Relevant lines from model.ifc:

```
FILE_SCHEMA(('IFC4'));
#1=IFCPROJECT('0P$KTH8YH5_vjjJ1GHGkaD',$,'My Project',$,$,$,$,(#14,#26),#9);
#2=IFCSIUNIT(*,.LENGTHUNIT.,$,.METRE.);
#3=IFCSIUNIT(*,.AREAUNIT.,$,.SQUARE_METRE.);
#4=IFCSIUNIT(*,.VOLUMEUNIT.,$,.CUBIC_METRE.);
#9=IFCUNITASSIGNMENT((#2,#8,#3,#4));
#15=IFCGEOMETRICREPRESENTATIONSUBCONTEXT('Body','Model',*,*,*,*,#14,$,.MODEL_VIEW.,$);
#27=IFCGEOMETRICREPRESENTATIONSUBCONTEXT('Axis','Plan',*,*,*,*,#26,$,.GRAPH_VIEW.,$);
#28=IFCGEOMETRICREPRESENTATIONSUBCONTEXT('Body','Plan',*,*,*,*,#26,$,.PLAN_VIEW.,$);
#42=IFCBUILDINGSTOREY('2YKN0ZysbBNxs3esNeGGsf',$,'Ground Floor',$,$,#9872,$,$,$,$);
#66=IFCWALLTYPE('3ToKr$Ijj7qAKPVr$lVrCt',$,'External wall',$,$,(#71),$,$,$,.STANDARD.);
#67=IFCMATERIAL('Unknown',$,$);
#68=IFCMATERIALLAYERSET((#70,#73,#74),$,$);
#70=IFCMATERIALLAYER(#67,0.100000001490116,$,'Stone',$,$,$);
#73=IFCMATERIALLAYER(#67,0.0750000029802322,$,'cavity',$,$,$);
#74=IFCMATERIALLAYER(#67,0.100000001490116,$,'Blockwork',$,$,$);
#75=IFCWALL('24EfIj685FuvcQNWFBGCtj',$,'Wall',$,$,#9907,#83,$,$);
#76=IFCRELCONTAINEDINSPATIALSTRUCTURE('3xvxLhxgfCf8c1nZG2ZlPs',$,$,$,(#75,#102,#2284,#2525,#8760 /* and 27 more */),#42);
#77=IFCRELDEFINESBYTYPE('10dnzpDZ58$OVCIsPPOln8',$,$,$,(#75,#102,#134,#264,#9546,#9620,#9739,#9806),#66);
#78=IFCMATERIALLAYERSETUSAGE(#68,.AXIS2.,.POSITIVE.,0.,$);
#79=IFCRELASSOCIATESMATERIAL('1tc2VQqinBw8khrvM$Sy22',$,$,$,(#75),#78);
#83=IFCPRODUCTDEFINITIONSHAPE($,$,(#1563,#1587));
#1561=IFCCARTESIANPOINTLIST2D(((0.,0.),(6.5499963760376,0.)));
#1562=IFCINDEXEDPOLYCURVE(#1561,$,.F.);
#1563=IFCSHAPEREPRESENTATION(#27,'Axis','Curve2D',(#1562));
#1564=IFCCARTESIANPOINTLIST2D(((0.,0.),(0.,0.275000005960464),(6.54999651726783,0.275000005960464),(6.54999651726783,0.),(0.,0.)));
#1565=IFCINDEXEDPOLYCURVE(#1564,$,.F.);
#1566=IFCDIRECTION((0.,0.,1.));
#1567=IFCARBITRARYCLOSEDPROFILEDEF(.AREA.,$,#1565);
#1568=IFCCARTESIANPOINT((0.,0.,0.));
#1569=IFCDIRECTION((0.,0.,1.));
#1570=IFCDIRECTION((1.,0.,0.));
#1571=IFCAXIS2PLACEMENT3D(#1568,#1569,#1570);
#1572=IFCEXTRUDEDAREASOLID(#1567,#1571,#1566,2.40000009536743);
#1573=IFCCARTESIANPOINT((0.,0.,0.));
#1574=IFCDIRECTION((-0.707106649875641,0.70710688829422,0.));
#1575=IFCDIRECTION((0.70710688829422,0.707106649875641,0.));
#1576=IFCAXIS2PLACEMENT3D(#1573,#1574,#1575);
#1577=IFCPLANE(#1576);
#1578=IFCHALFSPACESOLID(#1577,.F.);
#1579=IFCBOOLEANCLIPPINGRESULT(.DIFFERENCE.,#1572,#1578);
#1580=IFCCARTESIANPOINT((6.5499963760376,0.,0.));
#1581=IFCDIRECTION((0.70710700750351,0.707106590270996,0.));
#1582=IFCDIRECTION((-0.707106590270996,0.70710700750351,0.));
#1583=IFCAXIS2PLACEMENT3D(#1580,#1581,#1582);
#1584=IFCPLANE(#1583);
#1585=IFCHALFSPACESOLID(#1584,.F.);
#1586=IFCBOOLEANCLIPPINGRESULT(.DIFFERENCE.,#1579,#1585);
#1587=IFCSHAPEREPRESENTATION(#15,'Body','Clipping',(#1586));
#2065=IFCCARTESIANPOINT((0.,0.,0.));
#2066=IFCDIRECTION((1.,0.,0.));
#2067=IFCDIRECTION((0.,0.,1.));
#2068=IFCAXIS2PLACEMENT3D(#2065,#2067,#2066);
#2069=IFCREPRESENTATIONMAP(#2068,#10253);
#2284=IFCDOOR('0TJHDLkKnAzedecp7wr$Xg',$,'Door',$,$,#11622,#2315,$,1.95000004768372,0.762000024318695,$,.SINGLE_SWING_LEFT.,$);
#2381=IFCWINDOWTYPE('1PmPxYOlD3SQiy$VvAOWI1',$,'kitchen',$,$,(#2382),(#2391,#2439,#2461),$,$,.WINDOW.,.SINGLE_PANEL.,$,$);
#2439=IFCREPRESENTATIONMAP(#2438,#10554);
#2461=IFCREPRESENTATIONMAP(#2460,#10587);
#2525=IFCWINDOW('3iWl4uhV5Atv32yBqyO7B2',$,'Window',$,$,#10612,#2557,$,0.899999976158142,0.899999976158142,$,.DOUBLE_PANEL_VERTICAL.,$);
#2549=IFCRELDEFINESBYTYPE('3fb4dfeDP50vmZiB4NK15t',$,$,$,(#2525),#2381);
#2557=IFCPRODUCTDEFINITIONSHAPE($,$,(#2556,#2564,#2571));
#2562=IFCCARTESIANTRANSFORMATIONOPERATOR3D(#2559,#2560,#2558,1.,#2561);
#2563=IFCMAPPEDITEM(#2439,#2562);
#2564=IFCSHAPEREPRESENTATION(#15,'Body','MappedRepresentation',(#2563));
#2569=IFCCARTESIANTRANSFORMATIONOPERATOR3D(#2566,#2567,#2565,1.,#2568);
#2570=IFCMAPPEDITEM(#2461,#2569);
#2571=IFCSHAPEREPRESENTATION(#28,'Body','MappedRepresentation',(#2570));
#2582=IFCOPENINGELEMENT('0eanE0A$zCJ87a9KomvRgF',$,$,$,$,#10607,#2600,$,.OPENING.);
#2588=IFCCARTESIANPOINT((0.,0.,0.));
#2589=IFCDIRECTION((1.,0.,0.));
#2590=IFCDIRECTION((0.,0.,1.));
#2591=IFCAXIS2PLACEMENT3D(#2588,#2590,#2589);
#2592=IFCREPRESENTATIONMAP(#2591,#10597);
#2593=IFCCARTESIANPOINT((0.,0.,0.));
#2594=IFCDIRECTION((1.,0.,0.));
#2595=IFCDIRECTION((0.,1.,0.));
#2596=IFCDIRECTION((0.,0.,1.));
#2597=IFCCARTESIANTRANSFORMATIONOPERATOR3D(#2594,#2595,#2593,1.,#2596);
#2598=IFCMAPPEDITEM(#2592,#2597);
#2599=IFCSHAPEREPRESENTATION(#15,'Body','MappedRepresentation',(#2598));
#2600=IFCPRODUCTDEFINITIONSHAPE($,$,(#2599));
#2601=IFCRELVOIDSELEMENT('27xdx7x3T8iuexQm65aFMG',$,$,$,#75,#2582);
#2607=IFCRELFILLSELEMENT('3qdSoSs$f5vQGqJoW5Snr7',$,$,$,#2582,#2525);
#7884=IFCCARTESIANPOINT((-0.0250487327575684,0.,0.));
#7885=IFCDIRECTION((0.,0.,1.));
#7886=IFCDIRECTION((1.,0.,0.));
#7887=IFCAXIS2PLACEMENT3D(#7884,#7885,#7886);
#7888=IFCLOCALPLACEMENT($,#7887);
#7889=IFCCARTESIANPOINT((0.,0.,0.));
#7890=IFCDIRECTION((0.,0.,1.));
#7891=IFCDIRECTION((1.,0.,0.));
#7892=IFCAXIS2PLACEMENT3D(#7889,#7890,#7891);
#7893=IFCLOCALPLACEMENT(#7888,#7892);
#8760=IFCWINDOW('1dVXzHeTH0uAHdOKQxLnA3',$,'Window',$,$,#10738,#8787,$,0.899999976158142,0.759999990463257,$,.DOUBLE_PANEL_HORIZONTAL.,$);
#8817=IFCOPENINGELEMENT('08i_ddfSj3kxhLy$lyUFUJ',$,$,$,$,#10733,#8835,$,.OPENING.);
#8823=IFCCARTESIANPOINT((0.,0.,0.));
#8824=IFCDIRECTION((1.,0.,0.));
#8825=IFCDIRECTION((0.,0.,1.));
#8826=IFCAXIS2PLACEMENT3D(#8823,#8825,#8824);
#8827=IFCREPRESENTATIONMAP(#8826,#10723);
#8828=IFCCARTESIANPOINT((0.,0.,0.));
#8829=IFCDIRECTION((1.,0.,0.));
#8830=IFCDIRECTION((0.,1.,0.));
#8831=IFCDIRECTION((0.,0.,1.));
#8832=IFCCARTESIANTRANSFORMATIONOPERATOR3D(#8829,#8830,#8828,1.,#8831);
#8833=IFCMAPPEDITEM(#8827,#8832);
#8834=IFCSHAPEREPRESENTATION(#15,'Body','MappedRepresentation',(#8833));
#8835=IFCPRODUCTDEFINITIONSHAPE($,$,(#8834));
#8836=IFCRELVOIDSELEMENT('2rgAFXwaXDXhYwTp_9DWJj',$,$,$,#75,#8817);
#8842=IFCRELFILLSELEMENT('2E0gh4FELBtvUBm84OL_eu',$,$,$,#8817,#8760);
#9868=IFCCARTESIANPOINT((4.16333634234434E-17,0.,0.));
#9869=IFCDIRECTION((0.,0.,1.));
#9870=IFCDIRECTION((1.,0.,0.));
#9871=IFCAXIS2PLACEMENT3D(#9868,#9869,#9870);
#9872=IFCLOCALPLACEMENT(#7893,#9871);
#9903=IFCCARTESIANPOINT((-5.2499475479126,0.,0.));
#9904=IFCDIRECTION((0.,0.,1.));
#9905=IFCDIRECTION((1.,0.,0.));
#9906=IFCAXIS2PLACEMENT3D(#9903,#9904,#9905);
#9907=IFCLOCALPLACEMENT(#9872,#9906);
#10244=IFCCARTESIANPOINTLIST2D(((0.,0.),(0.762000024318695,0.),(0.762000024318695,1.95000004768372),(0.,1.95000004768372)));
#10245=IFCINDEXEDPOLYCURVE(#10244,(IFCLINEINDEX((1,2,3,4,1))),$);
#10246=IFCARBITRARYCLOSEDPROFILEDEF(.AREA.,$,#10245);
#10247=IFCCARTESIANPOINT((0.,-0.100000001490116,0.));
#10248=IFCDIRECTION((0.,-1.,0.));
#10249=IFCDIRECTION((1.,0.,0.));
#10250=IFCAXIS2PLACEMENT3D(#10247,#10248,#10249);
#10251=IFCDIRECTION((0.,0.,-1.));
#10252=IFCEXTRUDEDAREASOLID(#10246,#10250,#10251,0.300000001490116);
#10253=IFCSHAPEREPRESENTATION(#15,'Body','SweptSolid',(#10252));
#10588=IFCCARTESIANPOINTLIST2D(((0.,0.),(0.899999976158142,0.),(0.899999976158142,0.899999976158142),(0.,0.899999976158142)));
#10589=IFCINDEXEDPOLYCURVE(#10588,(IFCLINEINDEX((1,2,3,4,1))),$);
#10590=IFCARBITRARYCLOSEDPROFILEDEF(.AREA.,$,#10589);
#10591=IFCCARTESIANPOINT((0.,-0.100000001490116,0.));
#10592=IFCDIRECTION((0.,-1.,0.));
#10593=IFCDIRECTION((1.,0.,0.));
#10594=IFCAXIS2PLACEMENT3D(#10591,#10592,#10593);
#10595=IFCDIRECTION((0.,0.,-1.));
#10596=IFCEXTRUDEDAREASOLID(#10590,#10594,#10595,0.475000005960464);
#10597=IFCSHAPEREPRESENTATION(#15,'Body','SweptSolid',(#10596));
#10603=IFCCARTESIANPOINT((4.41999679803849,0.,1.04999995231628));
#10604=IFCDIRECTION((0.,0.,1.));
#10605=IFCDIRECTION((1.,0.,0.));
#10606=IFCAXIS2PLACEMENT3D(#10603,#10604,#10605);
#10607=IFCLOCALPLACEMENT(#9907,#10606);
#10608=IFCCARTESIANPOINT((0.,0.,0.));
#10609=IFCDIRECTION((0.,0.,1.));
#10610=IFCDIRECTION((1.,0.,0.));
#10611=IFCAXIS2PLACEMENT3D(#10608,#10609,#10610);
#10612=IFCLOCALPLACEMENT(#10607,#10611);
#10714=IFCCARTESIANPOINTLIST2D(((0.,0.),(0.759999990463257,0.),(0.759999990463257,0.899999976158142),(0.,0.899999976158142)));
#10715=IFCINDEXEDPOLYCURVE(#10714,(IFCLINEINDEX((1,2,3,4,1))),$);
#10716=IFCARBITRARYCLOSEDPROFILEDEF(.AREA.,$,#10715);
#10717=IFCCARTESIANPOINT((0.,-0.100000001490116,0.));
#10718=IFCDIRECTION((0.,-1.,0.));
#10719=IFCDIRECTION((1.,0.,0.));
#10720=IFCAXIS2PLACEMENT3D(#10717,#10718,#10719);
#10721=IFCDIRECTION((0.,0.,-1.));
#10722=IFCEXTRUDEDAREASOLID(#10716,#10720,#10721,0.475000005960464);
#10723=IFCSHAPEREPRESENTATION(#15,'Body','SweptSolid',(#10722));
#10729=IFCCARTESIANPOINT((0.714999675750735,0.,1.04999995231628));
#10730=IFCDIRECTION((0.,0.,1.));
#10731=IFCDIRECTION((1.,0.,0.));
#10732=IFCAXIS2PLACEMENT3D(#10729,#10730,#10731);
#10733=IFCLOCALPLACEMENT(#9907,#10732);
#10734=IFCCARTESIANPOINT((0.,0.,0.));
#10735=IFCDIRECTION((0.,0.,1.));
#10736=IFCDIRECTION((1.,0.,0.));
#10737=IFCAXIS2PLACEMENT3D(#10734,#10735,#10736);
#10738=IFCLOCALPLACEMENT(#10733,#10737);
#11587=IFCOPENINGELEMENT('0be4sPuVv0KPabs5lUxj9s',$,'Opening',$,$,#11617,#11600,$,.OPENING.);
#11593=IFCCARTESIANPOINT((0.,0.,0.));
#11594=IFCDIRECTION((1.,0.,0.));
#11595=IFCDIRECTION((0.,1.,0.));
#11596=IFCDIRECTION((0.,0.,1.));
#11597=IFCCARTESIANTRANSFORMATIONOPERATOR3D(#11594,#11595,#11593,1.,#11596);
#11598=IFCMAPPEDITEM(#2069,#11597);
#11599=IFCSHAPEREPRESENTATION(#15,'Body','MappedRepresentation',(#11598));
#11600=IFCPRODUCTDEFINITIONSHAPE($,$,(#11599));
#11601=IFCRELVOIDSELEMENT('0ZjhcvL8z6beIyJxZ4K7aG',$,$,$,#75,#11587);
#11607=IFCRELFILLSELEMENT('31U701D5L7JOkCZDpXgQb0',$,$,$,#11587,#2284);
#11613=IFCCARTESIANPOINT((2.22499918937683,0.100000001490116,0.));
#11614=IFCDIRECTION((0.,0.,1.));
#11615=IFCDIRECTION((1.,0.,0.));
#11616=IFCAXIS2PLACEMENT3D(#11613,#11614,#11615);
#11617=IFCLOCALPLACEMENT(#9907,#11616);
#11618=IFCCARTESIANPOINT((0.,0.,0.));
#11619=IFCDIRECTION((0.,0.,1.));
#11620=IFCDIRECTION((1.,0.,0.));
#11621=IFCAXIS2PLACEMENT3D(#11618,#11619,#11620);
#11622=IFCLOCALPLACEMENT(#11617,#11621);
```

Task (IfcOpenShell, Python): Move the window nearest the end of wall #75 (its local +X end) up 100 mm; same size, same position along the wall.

```python
import numpy as np
import ifcopenshell
import ifcopenshell.api.geometry
import ifcopenshell.util.placement
import ifcopenshell.util.unit

model = ifcopenshell.open("model.ifc")
unit_scale = ifcopenshell.util.unit.calculate_unit_scale(model)

window = model.by_guid("3iWl4uhV5Atv32yBqyO7B2")
opening = window.FillsVoids[0].RelatingOpeningElement
dz = 0.1 / unit_scale

shift = np.array([0.0, 0.0, dz])
# The window is placed relative to its opening, so it follows when the opening moves.
matrix = ifcopenshell.util.placement.get_local_placement(opening.ObjectPlacement)
matrix[:3, 3] += shift
ifcopenshell.api.geometry.edit_object_placement(
    model, product=opening, matrix=matrix, is_si=False, should_transform_children=True
)

print(f"moved by {dz * unit_scale:+.3f} m")

model.write("model_updated.ifc")
```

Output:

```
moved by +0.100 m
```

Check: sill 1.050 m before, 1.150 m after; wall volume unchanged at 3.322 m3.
